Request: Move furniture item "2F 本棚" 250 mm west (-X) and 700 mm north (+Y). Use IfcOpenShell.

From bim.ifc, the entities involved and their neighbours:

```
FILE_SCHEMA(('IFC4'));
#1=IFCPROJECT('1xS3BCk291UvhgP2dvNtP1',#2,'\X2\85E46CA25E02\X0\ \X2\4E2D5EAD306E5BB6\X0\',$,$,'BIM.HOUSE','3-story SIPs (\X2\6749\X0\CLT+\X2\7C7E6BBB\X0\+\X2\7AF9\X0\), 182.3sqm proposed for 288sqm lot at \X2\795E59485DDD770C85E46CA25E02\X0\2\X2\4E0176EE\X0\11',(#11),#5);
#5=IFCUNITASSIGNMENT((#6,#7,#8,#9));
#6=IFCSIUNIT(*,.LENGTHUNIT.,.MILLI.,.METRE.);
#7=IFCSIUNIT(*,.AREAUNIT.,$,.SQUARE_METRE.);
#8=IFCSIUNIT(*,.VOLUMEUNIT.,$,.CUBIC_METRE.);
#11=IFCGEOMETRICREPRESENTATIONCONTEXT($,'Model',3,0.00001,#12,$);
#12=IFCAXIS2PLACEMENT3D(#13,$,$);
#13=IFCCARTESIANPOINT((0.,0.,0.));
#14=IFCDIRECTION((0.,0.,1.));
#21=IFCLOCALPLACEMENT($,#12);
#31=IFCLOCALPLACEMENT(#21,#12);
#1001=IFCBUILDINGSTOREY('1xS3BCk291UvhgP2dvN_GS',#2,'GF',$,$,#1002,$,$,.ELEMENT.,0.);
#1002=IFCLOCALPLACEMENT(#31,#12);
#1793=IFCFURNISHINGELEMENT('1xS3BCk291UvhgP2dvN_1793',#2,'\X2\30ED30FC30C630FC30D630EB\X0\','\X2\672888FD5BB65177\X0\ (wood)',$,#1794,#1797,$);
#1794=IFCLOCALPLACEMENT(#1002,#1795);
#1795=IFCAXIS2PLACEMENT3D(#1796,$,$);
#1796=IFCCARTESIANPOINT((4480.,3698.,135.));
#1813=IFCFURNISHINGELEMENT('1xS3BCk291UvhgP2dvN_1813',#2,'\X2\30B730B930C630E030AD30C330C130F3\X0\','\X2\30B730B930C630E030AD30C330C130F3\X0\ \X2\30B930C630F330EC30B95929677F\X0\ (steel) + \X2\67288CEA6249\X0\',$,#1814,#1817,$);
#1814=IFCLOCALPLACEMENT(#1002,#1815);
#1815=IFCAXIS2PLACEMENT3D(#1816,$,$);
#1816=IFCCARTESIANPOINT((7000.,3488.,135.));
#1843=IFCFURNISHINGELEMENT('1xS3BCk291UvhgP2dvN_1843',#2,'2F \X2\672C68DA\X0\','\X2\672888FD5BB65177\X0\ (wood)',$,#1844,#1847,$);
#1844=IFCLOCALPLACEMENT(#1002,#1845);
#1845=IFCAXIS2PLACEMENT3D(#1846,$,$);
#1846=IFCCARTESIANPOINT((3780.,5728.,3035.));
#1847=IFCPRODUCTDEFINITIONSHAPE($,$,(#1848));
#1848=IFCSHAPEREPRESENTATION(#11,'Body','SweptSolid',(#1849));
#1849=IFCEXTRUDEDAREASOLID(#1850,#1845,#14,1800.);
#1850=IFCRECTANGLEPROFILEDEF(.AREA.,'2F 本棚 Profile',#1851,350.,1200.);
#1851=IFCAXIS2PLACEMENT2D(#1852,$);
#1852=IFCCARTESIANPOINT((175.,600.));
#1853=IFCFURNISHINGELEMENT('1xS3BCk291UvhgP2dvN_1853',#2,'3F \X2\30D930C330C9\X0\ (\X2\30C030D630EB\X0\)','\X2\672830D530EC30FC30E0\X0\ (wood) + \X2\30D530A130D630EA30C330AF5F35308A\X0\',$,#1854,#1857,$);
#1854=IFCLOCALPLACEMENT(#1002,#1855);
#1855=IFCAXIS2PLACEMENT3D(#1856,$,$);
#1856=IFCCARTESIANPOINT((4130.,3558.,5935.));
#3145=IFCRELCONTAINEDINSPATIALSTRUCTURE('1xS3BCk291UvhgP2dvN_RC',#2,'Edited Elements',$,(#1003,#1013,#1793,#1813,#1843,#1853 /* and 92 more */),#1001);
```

```python
import ifcopenshell
import ifcopenshell.api.geometry
import ifcopenshell.util.placement
import ifcopenshell.util.unit

model = ifcopenshell.open("bim.ifc")
unit_scale = ifcopenshell.util.unit.calculate_unit_scale(model)

item = model.by_guid("1xS3BCk291UvhgP2dvN_1843")
matrix = ifcopenshell.util.placement.get_local_placement(item.ObjectPlacement)
matrix[0, 3] -= 0.25 / unit_scale
matrix[1, 3] += 0.7 / unit_scale
ifcopenshell.api.geometry.edit_object_placement(model, product=item, matrix=matrix, is_si=False)

print(ifcopenshell.util.placement.get_local_placement(item.ObjectPlacement).round(3) + 0.0)

model.write("bim_rev.ifc")
```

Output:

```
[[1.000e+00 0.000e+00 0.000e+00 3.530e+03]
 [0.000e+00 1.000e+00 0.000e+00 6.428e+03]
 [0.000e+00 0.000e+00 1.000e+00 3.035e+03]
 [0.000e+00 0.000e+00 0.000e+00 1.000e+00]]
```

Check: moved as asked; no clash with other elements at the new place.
